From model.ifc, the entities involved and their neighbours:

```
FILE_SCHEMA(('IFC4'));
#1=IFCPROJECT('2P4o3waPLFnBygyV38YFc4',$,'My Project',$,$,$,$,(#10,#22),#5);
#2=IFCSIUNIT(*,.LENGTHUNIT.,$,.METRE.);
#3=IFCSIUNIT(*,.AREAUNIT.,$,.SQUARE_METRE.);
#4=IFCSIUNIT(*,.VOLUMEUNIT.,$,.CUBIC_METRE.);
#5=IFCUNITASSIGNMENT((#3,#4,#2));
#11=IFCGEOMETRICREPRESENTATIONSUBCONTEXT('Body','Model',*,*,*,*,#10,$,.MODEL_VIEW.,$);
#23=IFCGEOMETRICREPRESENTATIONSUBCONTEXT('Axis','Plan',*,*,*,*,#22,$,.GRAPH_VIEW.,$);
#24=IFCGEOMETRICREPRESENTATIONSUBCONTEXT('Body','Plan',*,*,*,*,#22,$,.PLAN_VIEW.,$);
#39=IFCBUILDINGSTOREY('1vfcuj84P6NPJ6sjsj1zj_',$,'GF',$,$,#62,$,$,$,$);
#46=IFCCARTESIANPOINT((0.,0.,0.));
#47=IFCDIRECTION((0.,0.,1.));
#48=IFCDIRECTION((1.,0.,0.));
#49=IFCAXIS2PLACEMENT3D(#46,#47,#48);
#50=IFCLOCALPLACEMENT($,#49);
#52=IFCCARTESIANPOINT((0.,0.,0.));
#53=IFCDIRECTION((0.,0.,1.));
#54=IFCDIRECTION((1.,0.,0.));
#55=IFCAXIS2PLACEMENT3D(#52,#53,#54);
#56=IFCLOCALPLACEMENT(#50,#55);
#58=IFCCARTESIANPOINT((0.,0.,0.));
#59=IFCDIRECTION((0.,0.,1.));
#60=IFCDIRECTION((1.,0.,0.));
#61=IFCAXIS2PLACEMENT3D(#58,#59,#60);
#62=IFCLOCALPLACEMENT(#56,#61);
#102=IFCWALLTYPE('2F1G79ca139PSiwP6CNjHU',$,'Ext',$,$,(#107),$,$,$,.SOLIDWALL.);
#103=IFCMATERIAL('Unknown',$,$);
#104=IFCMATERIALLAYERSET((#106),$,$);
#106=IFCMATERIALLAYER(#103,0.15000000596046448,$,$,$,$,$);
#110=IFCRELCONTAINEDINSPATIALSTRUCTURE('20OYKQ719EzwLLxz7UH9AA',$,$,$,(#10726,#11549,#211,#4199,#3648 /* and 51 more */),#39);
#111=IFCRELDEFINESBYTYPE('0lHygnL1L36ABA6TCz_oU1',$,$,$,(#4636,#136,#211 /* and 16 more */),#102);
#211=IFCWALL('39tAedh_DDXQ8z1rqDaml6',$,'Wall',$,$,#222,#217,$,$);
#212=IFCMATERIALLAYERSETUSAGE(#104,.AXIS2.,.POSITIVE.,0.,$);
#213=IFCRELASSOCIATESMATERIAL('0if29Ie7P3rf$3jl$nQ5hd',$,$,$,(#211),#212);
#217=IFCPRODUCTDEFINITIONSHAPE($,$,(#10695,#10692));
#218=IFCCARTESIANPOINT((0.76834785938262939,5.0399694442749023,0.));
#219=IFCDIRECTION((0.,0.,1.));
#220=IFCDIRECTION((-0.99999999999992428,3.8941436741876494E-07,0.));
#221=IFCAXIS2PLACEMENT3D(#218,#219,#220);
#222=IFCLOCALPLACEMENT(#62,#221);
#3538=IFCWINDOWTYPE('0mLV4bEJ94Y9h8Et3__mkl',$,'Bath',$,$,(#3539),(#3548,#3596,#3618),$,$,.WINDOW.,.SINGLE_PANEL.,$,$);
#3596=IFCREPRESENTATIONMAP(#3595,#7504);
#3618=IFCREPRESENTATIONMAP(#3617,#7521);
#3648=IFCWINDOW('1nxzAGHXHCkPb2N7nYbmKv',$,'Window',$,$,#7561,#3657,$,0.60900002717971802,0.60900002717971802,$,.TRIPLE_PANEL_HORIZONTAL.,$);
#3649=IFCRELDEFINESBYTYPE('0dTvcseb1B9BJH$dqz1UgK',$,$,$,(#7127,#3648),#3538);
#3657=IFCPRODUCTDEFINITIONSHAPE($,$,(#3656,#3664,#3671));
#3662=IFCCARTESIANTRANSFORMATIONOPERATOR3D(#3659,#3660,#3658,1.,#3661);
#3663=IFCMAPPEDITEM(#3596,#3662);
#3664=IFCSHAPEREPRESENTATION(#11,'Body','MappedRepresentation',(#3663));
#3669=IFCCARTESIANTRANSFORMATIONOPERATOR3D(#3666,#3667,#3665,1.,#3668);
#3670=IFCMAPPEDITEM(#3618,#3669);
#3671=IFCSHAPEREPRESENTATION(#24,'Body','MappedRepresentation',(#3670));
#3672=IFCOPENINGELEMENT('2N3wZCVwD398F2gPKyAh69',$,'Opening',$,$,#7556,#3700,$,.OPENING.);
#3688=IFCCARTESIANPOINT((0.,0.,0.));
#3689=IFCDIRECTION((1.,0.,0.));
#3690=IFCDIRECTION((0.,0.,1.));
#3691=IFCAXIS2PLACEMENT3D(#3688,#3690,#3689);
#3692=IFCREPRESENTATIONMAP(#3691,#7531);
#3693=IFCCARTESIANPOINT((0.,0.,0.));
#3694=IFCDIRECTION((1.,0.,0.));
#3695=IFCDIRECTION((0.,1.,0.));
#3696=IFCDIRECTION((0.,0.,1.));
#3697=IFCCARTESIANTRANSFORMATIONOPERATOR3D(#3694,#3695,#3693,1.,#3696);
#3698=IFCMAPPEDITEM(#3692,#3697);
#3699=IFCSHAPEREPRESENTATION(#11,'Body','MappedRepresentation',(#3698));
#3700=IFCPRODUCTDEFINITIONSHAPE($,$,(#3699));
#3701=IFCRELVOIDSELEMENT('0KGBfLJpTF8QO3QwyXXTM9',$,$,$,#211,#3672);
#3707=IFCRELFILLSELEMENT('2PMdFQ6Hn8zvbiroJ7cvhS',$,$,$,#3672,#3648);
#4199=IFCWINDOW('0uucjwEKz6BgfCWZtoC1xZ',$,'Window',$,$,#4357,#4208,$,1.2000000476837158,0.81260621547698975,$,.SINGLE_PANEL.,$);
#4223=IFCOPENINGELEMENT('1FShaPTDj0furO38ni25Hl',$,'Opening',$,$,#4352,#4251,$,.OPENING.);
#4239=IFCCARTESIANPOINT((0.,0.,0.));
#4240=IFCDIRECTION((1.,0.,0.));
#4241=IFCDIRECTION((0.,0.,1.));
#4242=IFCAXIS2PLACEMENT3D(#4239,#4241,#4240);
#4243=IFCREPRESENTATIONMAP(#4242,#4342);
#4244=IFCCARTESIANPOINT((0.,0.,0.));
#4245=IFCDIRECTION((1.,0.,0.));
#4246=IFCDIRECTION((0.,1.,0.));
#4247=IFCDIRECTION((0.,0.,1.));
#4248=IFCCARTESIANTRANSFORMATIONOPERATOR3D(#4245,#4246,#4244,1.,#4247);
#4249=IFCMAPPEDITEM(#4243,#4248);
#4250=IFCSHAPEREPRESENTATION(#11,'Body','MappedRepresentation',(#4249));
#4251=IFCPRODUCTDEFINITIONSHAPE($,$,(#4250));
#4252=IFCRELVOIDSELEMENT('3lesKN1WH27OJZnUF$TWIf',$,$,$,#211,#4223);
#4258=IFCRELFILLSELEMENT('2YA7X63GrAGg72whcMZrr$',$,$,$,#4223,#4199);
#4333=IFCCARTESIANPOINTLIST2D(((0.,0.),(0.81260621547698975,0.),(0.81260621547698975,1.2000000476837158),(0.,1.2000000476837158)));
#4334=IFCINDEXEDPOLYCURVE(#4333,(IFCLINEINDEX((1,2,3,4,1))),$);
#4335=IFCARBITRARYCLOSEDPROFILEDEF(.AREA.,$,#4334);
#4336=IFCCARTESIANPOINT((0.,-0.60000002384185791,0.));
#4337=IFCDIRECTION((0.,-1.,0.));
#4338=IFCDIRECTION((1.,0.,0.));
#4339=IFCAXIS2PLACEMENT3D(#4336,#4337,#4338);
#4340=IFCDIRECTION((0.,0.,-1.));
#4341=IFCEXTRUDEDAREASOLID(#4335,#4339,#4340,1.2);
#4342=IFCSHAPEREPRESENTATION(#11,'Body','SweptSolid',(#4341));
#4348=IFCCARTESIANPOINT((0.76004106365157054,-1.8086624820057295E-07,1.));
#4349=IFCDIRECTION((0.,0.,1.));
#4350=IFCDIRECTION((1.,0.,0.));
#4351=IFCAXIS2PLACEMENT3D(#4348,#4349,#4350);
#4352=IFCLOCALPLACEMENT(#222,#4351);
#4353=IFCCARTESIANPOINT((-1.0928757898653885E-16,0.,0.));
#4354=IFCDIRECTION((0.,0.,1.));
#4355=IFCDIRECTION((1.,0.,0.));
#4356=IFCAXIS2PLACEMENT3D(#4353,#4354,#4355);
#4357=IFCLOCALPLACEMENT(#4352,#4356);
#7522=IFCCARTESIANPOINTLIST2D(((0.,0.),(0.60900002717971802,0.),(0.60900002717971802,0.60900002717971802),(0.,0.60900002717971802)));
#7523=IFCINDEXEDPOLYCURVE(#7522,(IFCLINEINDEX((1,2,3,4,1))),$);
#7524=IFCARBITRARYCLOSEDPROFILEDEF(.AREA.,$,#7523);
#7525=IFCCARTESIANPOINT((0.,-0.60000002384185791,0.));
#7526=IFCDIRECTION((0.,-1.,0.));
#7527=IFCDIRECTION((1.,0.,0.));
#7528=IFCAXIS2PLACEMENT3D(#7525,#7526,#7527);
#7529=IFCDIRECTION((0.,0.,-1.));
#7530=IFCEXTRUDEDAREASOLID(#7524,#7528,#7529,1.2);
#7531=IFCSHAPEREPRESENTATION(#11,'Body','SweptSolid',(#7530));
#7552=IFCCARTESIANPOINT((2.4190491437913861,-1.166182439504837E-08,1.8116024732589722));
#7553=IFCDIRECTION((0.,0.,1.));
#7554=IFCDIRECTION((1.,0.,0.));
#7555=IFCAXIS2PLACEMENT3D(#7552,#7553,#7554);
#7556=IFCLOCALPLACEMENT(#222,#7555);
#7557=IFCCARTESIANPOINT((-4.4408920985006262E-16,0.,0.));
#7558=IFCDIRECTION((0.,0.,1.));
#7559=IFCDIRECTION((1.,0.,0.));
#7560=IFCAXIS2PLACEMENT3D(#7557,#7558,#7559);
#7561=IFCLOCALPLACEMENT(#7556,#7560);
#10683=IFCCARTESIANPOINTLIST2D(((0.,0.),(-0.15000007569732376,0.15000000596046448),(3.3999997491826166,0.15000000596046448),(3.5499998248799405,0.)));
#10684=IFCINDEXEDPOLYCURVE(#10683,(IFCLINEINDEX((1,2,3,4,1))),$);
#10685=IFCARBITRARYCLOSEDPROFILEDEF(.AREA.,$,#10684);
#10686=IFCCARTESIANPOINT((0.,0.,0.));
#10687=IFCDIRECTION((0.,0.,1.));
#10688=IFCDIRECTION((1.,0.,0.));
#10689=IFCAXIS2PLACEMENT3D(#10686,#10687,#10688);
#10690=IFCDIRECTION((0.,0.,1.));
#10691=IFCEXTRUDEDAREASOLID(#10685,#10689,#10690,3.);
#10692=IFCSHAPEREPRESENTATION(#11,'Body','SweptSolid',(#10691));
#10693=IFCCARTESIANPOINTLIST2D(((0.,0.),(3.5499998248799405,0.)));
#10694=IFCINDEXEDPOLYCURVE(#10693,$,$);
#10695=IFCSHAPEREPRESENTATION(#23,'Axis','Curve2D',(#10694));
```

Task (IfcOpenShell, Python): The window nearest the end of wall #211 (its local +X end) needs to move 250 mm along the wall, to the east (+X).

```python
import ifcopenshell
import ifcopenshell.api.geometry
import ifcopenshell.util.placement

model = ifcopenshell.open("model.ifc")

window = model.by_id(3648)
opening = window.FillsVoids[0].RelatingOpeningElement
wall = opening.VoidsElements[0].RelatingBuildingElement

wall_matrix = ifcopenshell.util.placement.get_local_placement(wall.ObjectPlacement)
shift = wall_matrix[:3, 0] * -0.25
before = ifcopenshell.util.placement.get_local_placement(window.ObjectPlacement)[:3, 3].copy()

# The window is placed relative to its opening, so it follows when the opening moves.
matrix = ifcopenshell.util.placement.get_local_placement(opening.ObjectPlacement)
matrix[:3, 3] += shift
ifcopenshell.api.geometry.edit_object_placement(
    model, product=opening, matrix=matrix, is_si=False, should_transform_children=True
)

after = ifcopenshell.util.placement.get_local_placement(window.ObjectPlacement)[:3, 3]
print("window moved by", (after - before).round(3) + 0.0)

model.write("model_v2.ifc")
```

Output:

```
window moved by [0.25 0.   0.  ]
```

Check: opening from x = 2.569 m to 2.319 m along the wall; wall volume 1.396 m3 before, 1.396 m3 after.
